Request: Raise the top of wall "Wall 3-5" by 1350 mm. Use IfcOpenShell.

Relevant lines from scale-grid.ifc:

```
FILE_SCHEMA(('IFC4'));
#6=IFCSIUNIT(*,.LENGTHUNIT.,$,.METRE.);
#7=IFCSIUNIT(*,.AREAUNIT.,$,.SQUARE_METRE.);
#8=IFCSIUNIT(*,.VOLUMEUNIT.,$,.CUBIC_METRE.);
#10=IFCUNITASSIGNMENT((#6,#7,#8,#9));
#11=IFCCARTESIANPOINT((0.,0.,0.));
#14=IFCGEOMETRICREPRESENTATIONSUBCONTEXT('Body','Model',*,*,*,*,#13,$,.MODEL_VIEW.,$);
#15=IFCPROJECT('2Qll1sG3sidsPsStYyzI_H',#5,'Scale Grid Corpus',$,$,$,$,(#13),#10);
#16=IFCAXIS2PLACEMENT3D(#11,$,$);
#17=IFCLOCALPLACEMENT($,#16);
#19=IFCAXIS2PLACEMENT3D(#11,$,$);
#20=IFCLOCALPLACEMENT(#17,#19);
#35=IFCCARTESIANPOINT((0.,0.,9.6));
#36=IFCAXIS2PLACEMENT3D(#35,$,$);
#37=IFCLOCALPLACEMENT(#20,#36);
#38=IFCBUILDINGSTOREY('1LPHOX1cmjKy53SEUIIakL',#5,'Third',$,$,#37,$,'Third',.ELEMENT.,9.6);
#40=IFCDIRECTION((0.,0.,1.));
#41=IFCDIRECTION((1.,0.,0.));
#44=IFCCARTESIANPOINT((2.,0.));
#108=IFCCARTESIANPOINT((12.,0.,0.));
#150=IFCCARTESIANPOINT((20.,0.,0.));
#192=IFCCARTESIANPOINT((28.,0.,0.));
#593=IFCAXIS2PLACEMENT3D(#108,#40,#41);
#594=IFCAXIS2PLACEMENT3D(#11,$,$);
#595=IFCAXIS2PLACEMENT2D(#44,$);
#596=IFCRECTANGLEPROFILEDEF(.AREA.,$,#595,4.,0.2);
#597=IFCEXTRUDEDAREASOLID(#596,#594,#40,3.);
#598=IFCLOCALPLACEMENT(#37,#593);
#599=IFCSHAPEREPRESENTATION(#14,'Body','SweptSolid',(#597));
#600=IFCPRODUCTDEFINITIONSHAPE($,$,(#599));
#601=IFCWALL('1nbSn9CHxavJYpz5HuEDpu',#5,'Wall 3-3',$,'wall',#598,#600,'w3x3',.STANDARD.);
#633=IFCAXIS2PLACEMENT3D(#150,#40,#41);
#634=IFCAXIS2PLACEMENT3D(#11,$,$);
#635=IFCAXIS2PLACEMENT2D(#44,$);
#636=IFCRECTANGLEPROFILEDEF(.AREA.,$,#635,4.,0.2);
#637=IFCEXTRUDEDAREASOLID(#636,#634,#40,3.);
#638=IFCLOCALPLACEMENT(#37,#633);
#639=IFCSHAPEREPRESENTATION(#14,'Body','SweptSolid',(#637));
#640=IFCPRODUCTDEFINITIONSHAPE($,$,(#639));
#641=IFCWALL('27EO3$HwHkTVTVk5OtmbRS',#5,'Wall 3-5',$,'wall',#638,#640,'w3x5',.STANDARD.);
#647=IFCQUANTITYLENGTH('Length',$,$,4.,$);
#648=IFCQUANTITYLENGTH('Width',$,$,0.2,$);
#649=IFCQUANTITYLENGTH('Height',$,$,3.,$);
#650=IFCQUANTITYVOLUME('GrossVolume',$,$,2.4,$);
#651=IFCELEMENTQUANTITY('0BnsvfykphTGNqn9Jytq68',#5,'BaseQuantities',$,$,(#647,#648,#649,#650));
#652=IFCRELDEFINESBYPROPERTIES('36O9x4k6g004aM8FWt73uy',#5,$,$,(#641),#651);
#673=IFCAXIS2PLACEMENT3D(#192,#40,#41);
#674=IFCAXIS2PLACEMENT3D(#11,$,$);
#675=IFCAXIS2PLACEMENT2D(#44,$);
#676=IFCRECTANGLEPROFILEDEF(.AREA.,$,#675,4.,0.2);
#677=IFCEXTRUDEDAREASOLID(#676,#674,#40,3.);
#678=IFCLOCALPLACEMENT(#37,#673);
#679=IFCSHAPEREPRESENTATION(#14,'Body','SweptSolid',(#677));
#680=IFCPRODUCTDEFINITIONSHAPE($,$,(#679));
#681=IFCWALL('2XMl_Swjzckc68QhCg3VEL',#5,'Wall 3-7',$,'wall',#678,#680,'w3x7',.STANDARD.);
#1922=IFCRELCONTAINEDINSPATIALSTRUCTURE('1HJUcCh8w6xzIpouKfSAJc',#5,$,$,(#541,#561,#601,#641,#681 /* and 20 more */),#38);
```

```python
import ifcopenshell
import ifcopenshell.api.pset
import ifcopenshell.geom
import ifcopenshell.util.element
import ifcopenshell.util.representation
import ifcopenshell.util.shape
import ifcopenshell.util.unit

model = ifcopenshell.open("scale-grid.ifc")
unit_scale = ifcopenshell.util.unit.calculate_unit_scale(model)
volume_scale = ifcopenshell.util.unit.calculate_unit_scale(model, "VOLUMEUNIT")
settings = ifcopenshell.geom.settings()


def volume(element):
    """Net volume in cubic metres, openings subtracted."""
    shape = ifcopenshell.geom.create_shape(settings, element)
    return ifcopenshell.util.shape.get_volume(shape.geometry)


wall = model.by_id(641)
before = volume(wall)

body = ifcopenshell.util.representation.get_representation(wall, "Model", "Body")
solid = body.Items[0]
old_height = solid.Depth
solid.Depth += 1.35 / unit_scale
after = volume(wall)

# Update the stored height, areas and volumes.
qto = model.by_id(ifcopenshell.util.element.get_pset(wall, "BaseQuantities", should_inherit=False)["id"])
ifcopenshell.api.pset.edit_qto(model, qto=qto, properties={
    "Height": solid.Depth,
    "GrossVolume": ifcopenshell.util.element.get_pset(wall, "BaseQuantities", "GrossVolume") * solid.Depth / old_height,
})

print(f"height {old_height:g} -> {solid.Depth:g}, volume {before:.3f} -> {after:.3f} m3")

model.write("scale-grid_edited.ifc")
```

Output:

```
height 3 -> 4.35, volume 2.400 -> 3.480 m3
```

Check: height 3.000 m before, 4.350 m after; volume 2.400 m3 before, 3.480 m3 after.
